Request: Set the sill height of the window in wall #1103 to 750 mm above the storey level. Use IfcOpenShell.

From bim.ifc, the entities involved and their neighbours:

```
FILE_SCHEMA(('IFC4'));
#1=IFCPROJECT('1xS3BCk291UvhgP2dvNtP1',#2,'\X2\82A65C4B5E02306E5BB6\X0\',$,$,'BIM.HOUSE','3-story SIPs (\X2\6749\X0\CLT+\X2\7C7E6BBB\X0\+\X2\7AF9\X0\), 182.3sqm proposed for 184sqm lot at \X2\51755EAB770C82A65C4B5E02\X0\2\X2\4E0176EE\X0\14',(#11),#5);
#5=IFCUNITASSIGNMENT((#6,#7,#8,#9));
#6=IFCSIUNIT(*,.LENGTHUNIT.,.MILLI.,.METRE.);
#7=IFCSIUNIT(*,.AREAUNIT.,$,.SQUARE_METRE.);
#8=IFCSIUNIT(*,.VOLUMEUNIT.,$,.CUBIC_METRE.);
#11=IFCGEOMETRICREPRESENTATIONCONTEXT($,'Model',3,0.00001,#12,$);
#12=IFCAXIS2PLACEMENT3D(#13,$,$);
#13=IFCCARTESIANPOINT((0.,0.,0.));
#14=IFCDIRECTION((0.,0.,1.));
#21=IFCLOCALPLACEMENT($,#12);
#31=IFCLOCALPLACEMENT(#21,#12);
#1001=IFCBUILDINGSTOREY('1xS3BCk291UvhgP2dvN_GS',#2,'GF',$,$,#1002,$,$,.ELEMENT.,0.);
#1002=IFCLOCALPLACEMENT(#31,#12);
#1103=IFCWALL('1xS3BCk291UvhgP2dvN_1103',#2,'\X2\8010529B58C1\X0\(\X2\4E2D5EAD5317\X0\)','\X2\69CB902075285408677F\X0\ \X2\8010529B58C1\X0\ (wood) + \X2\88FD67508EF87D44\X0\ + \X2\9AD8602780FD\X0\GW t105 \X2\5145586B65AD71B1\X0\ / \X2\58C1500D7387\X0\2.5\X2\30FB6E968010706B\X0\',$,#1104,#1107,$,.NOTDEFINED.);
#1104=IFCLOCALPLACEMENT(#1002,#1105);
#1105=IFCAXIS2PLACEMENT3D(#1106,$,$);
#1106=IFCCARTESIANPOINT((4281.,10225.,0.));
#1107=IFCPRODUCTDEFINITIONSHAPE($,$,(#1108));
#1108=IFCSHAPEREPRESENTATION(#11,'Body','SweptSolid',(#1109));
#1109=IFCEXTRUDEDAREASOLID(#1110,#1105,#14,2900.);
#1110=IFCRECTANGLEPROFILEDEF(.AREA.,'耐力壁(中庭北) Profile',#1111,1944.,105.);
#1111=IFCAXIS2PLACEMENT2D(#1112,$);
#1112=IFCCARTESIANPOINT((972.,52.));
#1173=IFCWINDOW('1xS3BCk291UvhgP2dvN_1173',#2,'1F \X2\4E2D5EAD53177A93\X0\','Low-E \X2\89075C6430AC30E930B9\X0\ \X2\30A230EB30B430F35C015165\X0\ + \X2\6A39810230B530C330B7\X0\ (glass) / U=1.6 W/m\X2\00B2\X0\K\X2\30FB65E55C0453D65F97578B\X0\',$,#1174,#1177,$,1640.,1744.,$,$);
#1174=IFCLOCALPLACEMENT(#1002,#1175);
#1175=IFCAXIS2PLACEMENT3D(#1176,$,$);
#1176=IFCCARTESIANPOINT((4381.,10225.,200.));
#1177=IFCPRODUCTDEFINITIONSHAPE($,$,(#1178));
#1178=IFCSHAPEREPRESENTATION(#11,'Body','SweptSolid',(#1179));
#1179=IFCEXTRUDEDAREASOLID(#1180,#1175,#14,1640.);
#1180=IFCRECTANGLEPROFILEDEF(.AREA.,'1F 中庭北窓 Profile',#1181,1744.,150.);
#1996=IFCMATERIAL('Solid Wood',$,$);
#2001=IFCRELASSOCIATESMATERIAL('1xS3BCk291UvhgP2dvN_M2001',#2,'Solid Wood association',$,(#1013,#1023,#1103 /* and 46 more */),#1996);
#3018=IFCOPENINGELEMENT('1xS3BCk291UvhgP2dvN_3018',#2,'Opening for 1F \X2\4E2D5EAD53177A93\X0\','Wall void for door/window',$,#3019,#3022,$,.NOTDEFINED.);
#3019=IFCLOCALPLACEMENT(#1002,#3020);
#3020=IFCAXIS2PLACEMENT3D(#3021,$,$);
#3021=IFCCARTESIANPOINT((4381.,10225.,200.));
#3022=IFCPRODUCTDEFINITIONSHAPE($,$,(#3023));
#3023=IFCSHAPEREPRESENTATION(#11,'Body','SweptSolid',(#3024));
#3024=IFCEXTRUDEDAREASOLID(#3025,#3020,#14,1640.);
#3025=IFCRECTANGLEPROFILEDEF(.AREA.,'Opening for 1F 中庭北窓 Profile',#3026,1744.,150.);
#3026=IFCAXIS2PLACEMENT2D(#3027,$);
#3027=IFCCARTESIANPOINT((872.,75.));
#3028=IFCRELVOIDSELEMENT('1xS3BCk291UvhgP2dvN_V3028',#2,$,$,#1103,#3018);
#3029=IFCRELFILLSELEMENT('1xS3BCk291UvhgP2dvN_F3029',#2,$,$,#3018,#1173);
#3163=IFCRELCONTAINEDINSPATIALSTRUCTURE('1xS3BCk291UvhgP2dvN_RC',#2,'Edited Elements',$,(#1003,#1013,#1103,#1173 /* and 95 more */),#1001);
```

```python
import numpy as np
import ifcopenshell
import ifcopenshell.api.geometry
import ifcopenshell.geom
import ifcopenshell.util.element
import ifcopenshell.util.placement
import ifcopenshell.util.shape
import ifcopenshell.util.unit

model = ifcopenshell.open("bim.ifc")
unit_scale = ifcopenshell.util.unit.calculate_unit_scale(model)

window = model.by_guid("1xS3BCk291UvhgP2dvN_1173")
opening = window.FillsVoids[0].RelatingOpeningElement
storey = ifcopenshell.util.element.get_container(window, ifc_class="IfcBuildingStorey")
level = ifcopenshell.util.placement.get_local_placement(storey.ObjectPlacement)[2, 3]

# The opening's origin need not be at the sill, so measure its lowest point.
shape = ifcopenshell.geom.create_shape(ifcopenshell.geom.settings(), opening)
bottom = ifcopenshell.util.shape.get_shape_bottom_elevation(shape, shape.geometry) / unit_scale
dz = level + 0.75 / unit_scale - bottom

shift = np.array([0.0, 0.0, dz])
# The window is not placed relative to its opening, so move both.
for product in (opening, window):
    matrix = ifcopenshell.util.placement.get_local_placement(product.ObjectPlacement)
    matrix[:3, 3] += shift
    ifcopenshell.api.geometry.edit_object_placement(model, product=product, matrix=matrix, is_si=False)

print(f"moved by {dz * unit_scale:+.3f} m")

model.write("bim_updated.ifc")
```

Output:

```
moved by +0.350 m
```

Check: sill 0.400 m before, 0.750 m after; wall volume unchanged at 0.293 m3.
